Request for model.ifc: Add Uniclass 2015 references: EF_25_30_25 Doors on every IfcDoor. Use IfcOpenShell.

First a look at what the model holds.

```python
import ifcopenshell

model = ifcopenshell.open("model.ifc")
print(model.schema)
print("classifications:", [c.Name for c in model.by_type("IfcClassification")])
for ifc_class in ("IfcDoor", "IfcRoof", "IfcStair", "IfcWall", "IfcWindow"):
    print(ifc_class, len(model.by_type(ifc_class)))
```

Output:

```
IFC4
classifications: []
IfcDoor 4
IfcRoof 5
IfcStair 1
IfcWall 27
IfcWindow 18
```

```python
import ifcopenshell
import ifcopenshell.api.classification

model = ifcopenshell.open("model.ifc")

system = ifcopenshell.api.classification.add_classification(model, classification="Uniclass 2015")

codes = {
    "IfcDoor": ("EF_25_30_25", "Doors"),
}
for ifc_class, (code, name) in codes.items():
    products = model.by_type(ifc_class)
    ifcopenshell.api.classification.add_reference(
        model, products=products, classification=system, identification=code, name=name
    )
    print(code, len(products))

model.write("model_edited.ifc")
```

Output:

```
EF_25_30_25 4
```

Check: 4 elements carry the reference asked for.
